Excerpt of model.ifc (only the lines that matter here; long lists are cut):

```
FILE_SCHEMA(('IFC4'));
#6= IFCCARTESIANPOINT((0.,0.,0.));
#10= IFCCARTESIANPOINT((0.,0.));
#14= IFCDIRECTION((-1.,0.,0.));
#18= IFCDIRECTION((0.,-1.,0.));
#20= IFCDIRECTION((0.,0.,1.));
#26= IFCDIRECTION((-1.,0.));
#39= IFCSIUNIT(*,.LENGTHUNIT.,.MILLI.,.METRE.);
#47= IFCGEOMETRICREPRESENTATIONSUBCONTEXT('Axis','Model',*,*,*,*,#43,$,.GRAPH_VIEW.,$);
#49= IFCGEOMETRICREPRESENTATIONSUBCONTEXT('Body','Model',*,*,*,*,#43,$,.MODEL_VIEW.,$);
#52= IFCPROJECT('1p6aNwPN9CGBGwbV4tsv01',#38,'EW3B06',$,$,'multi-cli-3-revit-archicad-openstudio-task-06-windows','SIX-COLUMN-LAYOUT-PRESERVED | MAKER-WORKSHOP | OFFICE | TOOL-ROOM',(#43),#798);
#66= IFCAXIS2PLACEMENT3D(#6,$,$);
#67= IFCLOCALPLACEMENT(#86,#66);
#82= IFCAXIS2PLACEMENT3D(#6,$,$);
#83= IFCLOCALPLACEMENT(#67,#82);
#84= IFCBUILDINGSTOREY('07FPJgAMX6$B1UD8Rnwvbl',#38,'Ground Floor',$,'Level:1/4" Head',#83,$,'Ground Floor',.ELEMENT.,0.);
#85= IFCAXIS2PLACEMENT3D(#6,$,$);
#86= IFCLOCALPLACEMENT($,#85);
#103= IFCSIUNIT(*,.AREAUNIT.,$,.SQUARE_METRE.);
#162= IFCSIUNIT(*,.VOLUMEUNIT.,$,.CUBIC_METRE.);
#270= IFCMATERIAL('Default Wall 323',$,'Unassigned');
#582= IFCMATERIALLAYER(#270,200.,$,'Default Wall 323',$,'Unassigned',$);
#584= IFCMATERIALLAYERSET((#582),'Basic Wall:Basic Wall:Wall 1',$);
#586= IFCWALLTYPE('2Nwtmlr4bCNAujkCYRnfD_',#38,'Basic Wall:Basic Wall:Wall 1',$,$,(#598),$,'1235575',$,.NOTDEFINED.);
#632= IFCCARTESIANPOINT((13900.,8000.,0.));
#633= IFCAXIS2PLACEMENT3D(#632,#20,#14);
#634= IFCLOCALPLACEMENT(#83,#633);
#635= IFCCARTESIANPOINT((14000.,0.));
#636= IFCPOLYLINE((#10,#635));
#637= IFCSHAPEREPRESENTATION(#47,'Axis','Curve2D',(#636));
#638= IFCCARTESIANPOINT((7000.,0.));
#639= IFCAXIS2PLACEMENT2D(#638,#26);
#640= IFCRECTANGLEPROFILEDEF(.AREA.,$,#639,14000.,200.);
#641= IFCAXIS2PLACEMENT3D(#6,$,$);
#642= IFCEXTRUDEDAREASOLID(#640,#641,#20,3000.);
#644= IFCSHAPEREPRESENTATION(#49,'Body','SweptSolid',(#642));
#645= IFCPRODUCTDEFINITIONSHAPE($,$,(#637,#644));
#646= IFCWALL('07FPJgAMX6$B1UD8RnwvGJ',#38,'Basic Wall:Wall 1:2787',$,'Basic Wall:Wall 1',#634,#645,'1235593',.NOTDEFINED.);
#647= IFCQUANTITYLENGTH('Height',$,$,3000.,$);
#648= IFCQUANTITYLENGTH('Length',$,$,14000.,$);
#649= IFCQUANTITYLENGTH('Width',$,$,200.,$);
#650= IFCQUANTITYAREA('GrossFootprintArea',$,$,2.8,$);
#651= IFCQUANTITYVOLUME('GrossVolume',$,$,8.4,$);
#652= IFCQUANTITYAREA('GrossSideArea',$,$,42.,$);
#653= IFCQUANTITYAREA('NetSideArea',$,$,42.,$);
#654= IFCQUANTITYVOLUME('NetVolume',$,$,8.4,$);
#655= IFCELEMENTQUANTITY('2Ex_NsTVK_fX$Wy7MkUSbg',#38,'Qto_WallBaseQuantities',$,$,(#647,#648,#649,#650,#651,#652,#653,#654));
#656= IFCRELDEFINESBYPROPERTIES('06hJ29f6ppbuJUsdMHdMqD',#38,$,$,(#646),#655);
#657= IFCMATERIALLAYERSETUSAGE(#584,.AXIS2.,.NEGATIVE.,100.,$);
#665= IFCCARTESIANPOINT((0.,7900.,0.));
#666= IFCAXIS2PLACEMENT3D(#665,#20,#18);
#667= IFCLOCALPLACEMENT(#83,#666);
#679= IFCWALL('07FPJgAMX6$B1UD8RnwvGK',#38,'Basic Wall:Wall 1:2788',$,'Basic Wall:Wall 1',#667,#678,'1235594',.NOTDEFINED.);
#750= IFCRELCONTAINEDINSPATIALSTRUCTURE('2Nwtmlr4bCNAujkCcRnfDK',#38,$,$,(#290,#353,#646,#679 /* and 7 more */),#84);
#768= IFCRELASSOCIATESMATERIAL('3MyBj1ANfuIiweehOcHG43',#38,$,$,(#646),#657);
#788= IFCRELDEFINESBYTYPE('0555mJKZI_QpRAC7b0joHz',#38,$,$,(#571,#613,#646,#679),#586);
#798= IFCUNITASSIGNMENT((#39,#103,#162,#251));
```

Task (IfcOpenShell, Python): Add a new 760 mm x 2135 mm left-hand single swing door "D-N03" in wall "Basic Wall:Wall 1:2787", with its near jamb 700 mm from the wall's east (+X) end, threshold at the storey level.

```python
import numpy as np
import ifcopenshell
import ifcopenshell.api.feature
import ifcopenshell.api.geometry
import ifcopenshell.api.pset
import ifcopenshell.api.root
import ifcopenshell.api.spatial
import ifcopenshell.geom
import ifcopenshell.util.element
import ifcopenshell.util.placement
import ifcopenshell.util.representation
import ifcopenshell.util.shape
import ifcopenshell.util.unit

model = ifcopenshell.open("model.ifc")
unit_scale = ifcopenshell.util.unit.calculate_unit_scale(model)
area_scale = ifcopenshell.util.unit.calculate_unit_scale(model, "AREAUNIT")
volume_scale = ifcopenshell.util.unit.calculate_unit_scale(model, "VOLUMEUNIT")
settings = ifcopenshell.geom.settings()


def volume(element):
    """Net volume in cubic metres, openings subtracted."""
    shape = ifcopenshell.geom.create_shape(settings, element)
    return ifcopenshell.util.shape.get_volume(shape.geometry)


wall = model.by_guid("07FPJgAMX6$B1UD8RnwvGJ")
storey = ifcopenshell.util.element.get_container(wall, ifc_class="IfcBuildingStorey")
context = ifcopenshell.util.representation.get_context(model, "Model", "Body", "MODEL_VIEW")
before = volume(wall)

width, height, from_end, sill = 0.76, 2.135, 0.7, 0.0  # metres

# The wall runs along its own X axis, and the end named is its -X end.
wall_shape = ifcopenshell.geom.create_shape(settings, wall)
x, y, z = ifcopenshell.util.shape.get_vertices(wall_shape.geometry).T
start = x.min() + from_end
face, thickness = float(y.min()), float(y.max() - y.min())
wall_matrix = ifcopenshell.util.placement.get_local_placement(wall.ObjectPlacement)
level = ifcopenshell.util.placement.get_local_placement(storey.ObjectPlacement)[2, 3]


def in_wall(x, y):
    """Placement at x, y metres in the wall's axes, at sill height."""
    matrix = wall_matrix.copy()
    matrix[:, 3] = wall_matrix @ np.array([x / unit_scale, y / unit_scale, 0.0, 1.0])
    matrix[2, 3] = level + sill / unit_scale
    return matrix


# Opening: a box that overshoots both wall faces by 50 mm.
opening = ifcopenshell.api.root.create_entity(model, ifc_class="IfcOpeningElement", predefined_type="OPENING")
box = ifcopenshell.api.geometry.add_wall_representation(
    model, context=context, length=width, height=height, thickness=thickness + 0.1
)
ifcopenshell.api.geometry.assign_representation(model, product=opening, representation=box)
ifcopenshell.api.geometry.edit_object_placement(model, product=opening, matrix=in_wall(start, face - 0.05), is_si=False)
ifcopenshell.api.feature.add_feature(model, feature=opening, element=wall)

door = ifcopenshell.api.root.create_entity(model, ifc_class="IfcDoor", name="D-N03", predefined_type="DOOR")
door.OverallWidth, door.OverallHeight = width / unit_scale, height / unit_scale
door.OperationType = "SINGLE_SWING_LEFT"
body = ifcopenshell.api.geometry.add_door_representation(
    model,
    context=context,
    overall_width=door.OverallWidth,
    overall_height=door.OverallHeight,
    operation_type="SINGLE_SWING_LEFT",
    lining_properties={"LiningDepth": thickness / unit_scale, "ThresholdDepth": thickness / unit_scale},
)
ifcopenshell.api.geometry.assign_representation(model, product=door, representation=body)
ifcopenshell.api.spatial.assign_container(model, products=[door], relating_structure=storey)
ifcopenshell.api.feature.add_filling(model, opening=opening, element=door)

# The lining spans the wall, so the door starts at the wall face.
ifcopenshell.api.geometry.edit_object_placement(model, product=door, matrix=in_wall(start, face), is_si=False)

after = volume(wall)

# Update the wall's stored quantities.
qto = model.by_id(ifcopenshell.util.element.get_pset(wall, "Qto_WallBaseQuantities", should_inherit=False)["id"])
ifcopenshell.api.pset.edit_qto(model, qto=qto, properties={
    "NetSideArea": after / thickness / area_scale,
    "NetVolume": after / volume_scale,
})

print(f"wall volume {before:.3f} -> {after:.3f} m3")

model.write("model-out.ifc")
```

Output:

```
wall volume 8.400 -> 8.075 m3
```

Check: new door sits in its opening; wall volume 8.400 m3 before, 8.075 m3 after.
